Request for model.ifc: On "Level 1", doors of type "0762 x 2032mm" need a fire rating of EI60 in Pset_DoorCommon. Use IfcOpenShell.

First a look at what the model holds.

```python
import ifcopenshell
import ifcopenshell.util.element

model = ifcopenshell.open("model.ifc")
print(model.schema)
storey = next(s for s in model.by_type("IfcBuildingStorey") if s.Name == "Level 1")
doors = [e for e in ifcopenshell.util.element.get_decomposition(storey) if e.is_a("IfcDoor")]
seen = {}
for e in doors:
    element_type = ifcopenshell.util.element.get_type(e)
    key = (element_type.Name if element_type != e and element_type else None, ifcopenshell.util.element.get_pset(e, "Pset_DoorCommon", "FireRating"))
    seen[key] = seen.get(key, 0) + 1
for (name, value), count in sorted(seen.items(), key=str):
    print(count, "x", name, "|", value)
```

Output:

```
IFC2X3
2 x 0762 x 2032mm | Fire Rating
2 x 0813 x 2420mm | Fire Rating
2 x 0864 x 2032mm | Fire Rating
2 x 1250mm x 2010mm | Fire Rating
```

```python
import ifcopenshell
import ifcopenshell.api.pset
import ifcopenshell.util.element

model = ifcopenshell.open("model.ifc")

storey = next(s for s in model.by_type("IfcBuildingStorey") if s.Name == "Level 1")
doors = [e for e in ifcopenshell.util.element.get_decomposition(storey) if e.is_a("IfcDoor")]

count = 0
for e in doors:
    element_type = ifcopenshell.util.element.get_type(e)
    if element_type in (None, e) or element_type.Name != "0762 x 2032mm":
        continue
    # add_pset returns the element's existing set when there is one.
    pset = ifcopenshell.api.pset.add_pset(model, product=e, name="Pset_DoorCommon")
    ifcopenshell.api.pset.edit_pset(model, pset=pset, properties={"FireRating": "EI60"})
    count += 1

print(count, "doors updated")

model.write("model_v2.ifc")
```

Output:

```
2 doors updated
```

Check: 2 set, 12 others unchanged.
